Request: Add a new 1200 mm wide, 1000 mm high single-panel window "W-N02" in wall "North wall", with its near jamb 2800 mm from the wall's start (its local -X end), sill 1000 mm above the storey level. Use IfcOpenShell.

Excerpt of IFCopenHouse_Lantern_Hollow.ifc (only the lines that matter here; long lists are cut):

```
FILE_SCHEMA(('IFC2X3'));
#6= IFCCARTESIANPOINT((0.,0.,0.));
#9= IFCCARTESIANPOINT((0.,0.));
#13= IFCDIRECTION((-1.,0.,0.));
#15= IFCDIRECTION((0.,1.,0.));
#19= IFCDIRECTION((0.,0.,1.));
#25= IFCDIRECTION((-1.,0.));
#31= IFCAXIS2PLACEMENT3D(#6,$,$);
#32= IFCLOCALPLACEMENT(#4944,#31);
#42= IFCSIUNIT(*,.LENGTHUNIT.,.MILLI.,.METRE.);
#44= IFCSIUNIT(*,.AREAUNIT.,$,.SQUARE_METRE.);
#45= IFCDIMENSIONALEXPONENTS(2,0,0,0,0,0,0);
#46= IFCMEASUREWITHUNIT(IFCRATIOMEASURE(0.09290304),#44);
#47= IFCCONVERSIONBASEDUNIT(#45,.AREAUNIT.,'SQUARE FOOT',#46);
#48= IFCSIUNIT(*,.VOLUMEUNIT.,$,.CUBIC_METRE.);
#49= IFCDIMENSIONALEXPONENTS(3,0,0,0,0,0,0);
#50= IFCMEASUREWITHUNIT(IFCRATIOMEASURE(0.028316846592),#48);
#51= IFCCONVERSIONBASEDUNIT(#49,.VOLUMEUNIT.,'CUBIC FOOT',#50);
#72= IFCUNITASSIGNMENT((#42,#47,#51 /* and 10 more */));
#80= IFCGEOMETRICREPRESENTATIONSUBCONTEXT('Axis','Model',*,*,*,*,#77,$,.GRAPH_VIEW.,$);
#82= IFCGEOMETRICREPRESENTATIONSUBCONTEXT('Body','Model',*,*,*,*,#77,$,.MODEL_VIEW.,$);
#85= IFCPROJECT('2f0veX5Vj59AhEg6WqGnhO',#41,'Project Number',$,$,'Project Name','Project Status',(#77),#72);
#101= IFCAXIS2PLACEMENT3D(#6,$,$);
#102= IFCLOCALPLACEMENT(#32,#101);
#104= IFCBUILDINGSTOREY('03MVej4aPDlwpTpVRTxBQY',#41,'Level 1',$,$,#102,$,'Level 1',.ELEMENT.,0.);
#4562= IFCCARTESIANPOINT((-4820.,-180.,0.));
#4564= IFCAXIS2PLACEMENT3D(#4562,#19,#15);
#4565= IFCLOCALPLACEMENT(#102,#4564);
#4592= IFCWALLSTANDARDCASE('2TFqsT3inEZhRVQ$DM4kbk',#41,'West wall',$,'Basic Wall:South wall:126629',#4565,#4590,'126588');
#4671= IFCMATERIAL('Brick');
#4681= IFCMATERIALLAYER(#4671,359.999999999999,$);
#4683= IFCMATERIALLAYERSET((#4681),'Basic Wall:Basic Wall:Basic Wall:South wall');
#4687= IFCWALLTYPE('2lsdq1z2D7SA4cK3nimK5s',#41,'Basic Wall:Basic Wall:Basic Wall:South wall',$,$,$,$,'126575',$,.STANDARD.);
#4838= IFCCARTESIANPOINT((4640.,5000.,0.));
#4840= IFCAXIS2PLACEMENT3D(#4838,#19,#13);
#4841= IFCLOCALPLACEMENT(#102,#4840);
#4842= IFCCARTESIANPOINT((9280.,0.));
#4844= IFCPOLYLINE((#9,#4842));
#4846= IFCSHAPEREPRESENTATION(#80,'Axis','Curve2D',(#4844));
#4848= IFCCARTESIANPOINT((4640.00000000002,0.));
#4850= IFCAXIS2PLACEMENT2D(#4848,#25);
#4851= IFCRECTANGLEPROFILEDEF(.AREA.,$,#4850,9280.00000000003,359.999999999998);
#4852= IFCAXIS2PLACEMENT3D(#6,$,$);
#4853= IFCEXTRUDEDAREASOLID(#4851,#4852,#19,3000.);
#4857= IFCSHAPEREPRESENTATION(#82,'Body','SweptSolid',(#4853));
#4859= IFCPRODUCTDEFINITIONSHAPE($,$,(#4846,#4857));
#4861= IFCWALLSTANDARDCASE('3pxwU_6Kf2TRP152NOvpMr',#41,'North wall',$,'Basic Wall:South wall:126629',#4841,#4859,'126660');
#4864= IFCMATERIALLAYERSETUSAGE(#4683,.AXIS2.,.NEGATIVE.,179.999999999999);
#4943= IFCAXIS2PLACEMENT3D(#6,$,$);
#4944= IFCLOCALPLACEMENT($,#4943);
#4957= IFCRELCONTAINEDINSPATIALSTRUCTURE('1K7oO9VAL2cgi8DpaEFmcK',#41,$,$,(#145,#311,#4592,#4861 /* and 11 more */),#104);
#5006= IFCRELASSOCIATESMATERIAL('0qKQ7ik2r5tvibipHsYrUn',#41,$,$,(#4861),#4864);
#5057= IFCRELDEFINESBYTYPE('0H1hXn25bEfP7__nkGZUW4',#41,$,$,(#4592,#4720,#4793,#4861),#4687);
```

```python
import numpy as np
import ifcopenshell
import ifcopenshell.api.feature
import ifcopenshell.api.geometry
import ifcopenshell.api.root
import ifcopenshell.api.spatial
import ifcopenshell.api.type
import ifcopenshell.geom
import ifcopenshell.util.element
import ifcopenshell.util.placement
import ifcopenshell.util.representation
import ifcopenshell.util.shape
import ifcopenshell.util.unit

model = ifcopenshell.open("IFCopenHouse_Lantern_Hollow.ifc")
unit_scale = ifcopenshell.util.unit.calculate_unit_scale(model)
settings = ifcopenshell.geom.settings()


def volume(element):
    """Net volume in cubic metres, openings subtracted."""
    shape = ifcopenshell.geom.create_shape(settings, element)
    return ifcopenshell.util.shape.get_volume(shape.geometry)


wall = model.by_guid("3pxwU_6Kf2TRP152NOvpMr")
storey = ifcopenshell.util.element.get_container(wall, ifc_class="IfcBuildingStorey")
context = ifcopenshell.util.representation.get_context(model, "Model", "Body", "MODEL_VIEW")
before = volume(wall)

width, height, from_end, sill = 1.2, 1, 2.8, 1  # metres

# The wall runs along its own X axis, and the end named is its -X end.
wall_shape = ifcopenshell.geom.create_shape(settings, wall)
x, y, z = ifcopenshell.util.shape.get_vertices(wall_shape.geometry).T
start = x.min() + from_end
face, thickness = float(y.min()), float(y.max() - y.min())
wall_matrix = ifcopenshell.util.placement.get_local_placement(wall.ObjectPlacement)
level = ifcopenshell.util.placement.get_local_placement(storey.ObjectPlacement)[2, 3]


def in_wall(x, y):
    """Placement at x, y metres in the wall's axes, at sill height."""
    matrix = wall_matrix.copy()
    matrix[:, 3] = wall_matrix @ np.array([x / unit_scale, y / unit_scale, 0.0, 1.0])
    matrix[2, 3] = level + sill / unit_scale
    return matrix


# Opening: a box that overshoots both wall faces by 50 mm.
opening = ifcopenshell.api.root.create_entity(model, ifc_class="IfcOpeningElement")
box = ifcopenshell.api.geometry.add_wall_representation(
    model, context=context, length=width, height=height, thickness=thickness + 0.1
)
ifcopenshell.api.geometry.assign_representation(model, product=opening, representation=box)
ifcopenshell.api.geometry.edit_object_placement(model, product=opening, matrix=in_wall(start, face - 0.05), is_si=False)
ifcopenshell.api.feature.add_feature(model, feature=opening, element=wall)

window = ifcopenshell.api.root.create_entity(model, ifc_class="IfcWindow", name="W-N02")
window.OverallWidth, window.OverallHeight = width / unit_scale, height / unit_scale
body = ifcopenshell.api.geometry.add_window_representation(
    model,
    context=context,
    overall_width=window.OverallWidth,
    overall_height=window.OverallHeight,
    partition_type="SINGLE_PANEL",
)
ifcopenshell.api.geometry.assign_representation(model, product=window, representation=body)
ifcopenshell.api.spatial.assign_container(model, products=[window], relating_structure=storey)
fills = ifcopenshell.api.feature.add_filling(model, opening=opening, element=window)
fills.OwnerHistory = window.OwnerHistory  # required in IFC2X3

# IFC2X3 keeps the operation on the window style.
style = ifcopenshell.api.root.create_entity(model, ifc_class="IfcWindowStyle", name="W-N02")
style.OperationType, style.ConstructionType = "SINGLE_PANEL", "NOTDEFINED"
style.ParameterTakesPrecedence = style.Sizeable = False
ifcopenshell.api.type.assign_type(model, related_objects=[window], relating_type=style)

# Centre the window in the wall's thickness.
ifcopenshell.api.geometry.edit_object_placement(model, product=window, matrix=in_wall(start, face), is_si=False)
window_shape = ifcopenshell.geom.create_shape(settings, window)
depth = ifcopenshell.util.shape.get_vertices(window_shape.geometry)[:, 1]
offset = face + thickness / 2 - (depth.min() + depth.max()) / 2
ifcopenshell.api.geometry.edit_object_placement(model, product=window, matrix=in_wall(start, offset), is_si=False)

after = volume(wall)

print(f"wall volume {before:.3f} -> {after:.3f} m3")

model.write("IFCopenHouse_Lantern_Hollow_updated.ifc")
```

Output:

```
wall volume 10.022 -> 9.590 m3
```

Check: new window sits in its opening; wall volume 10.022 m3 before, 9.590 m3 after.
